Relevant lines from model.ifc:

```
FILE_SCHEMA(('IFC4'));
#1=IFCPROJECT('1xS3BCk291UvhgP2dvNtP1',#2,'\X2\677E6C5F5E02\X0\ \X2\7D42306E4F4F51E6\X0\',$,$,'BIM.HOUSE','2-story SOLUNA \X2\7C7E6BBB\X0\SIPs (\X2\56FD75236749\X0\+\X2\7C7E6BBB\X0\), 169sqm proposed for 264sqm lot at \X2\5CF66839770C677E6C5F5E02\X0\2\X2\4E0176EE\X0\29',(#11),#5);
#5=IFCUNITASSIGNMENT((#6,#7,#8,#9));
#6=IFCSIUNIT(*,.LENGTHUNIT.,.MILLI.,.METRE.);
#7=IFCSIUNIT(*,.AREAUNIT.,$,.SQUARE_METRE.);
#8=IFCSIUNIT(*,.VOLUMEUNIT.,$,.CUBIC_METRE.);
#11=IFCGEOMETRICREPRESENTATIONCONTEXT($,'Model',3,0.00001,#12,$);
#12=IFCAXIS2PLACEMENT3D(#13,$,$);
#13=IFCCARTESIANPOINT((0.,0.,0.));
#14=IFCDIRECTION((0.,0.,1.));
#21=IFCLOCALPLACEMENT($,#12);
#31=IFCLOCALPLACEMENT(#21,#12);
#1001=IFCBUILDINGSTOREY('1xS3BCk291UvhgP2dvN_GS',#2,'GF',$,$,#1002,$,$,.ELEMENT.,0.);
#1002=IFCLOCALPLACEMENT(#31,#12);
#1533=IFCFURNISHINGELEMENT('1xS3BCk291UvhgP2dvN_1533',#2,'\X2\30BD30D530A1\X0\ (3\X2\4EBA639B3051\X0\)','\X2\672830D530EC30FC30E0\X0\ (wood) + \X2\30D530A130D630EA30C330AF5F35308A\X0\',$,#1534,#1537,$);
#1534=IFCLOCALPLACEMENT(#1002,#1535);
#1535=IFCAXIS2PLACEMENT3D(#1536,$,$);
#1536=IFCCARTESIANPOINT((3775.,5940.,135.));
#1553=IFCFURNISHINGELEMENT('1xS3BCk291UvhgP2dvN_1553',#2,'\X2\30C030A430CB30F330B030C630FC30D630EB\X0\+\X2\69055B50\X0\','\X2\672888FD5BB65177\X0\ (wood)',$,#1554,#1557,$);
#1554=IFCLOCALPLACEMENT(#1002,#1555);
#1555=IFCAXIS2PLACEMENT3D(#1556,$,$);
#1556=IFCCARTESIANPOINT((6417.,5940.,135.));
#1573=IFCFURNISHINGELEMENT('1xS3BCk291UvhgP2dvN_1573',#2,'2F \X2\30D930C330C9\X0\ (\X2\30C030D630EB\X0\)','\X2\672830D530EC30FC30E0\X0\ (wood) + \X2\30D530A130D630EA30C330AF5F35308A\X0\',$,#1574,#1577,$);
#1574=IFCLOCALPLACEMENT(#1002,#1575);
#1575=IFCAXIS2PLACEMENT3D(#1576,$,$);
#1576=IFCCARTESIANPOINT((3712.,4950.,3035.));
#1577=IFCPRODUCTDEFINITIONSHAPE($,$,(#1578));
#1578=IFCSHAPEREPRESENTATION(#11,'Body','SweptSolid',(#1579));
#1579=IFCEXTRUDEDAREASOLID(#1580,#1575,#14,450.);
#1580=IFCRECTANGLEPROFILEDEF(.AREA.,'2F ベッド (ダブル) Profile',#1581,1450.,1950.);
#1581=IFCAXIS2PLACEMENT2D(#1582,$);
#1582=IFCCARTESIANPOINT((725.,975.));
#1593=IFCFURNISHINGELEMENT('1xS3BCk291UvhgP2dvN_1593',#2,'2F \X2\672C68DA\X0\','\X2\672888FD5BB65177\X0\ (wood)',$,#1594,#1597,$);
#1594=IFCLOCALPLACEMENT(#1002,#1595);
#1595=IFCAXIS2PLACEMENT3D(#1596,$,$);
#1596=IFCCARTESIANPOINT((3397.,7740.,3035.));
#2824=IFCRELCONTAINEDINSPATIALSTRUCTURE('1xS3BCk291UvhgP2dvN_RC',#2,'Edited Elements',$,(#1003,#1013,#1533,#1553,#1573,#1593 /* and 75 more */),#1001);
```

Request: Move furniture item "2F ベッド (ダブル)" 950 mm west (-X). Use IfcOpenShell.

```python
import ifcopenshell
import ifcopenshell.api.geometry
import ifcopenshell.util.placement

model = ifcopenshell.open("model.ifc")

item = model.by_guid("1xS3BCk291UvhgP2dvN_1573")
matrix = ifcopenshell.util.placement.get_local_placement(item.ObjectPlacement)
matrix[0, 3] -= 950.0
ifcopenshell.api.geometry.edit_object_placement(model, product=item, matrix=matrix, is_si=False)

print(ifcopenshell.util.placement.get_local_placement(item.ObjectPlacement).round(3) + 0.0)

model.write("model_rev.ifc")
```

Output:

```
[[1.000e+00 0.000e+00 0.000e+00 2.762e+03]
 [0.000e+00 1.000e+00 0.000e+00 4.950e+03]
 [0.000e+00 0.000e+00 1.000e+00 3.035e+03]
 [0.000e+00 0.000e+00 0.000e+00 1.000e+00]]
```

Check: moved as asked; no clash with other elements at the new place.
